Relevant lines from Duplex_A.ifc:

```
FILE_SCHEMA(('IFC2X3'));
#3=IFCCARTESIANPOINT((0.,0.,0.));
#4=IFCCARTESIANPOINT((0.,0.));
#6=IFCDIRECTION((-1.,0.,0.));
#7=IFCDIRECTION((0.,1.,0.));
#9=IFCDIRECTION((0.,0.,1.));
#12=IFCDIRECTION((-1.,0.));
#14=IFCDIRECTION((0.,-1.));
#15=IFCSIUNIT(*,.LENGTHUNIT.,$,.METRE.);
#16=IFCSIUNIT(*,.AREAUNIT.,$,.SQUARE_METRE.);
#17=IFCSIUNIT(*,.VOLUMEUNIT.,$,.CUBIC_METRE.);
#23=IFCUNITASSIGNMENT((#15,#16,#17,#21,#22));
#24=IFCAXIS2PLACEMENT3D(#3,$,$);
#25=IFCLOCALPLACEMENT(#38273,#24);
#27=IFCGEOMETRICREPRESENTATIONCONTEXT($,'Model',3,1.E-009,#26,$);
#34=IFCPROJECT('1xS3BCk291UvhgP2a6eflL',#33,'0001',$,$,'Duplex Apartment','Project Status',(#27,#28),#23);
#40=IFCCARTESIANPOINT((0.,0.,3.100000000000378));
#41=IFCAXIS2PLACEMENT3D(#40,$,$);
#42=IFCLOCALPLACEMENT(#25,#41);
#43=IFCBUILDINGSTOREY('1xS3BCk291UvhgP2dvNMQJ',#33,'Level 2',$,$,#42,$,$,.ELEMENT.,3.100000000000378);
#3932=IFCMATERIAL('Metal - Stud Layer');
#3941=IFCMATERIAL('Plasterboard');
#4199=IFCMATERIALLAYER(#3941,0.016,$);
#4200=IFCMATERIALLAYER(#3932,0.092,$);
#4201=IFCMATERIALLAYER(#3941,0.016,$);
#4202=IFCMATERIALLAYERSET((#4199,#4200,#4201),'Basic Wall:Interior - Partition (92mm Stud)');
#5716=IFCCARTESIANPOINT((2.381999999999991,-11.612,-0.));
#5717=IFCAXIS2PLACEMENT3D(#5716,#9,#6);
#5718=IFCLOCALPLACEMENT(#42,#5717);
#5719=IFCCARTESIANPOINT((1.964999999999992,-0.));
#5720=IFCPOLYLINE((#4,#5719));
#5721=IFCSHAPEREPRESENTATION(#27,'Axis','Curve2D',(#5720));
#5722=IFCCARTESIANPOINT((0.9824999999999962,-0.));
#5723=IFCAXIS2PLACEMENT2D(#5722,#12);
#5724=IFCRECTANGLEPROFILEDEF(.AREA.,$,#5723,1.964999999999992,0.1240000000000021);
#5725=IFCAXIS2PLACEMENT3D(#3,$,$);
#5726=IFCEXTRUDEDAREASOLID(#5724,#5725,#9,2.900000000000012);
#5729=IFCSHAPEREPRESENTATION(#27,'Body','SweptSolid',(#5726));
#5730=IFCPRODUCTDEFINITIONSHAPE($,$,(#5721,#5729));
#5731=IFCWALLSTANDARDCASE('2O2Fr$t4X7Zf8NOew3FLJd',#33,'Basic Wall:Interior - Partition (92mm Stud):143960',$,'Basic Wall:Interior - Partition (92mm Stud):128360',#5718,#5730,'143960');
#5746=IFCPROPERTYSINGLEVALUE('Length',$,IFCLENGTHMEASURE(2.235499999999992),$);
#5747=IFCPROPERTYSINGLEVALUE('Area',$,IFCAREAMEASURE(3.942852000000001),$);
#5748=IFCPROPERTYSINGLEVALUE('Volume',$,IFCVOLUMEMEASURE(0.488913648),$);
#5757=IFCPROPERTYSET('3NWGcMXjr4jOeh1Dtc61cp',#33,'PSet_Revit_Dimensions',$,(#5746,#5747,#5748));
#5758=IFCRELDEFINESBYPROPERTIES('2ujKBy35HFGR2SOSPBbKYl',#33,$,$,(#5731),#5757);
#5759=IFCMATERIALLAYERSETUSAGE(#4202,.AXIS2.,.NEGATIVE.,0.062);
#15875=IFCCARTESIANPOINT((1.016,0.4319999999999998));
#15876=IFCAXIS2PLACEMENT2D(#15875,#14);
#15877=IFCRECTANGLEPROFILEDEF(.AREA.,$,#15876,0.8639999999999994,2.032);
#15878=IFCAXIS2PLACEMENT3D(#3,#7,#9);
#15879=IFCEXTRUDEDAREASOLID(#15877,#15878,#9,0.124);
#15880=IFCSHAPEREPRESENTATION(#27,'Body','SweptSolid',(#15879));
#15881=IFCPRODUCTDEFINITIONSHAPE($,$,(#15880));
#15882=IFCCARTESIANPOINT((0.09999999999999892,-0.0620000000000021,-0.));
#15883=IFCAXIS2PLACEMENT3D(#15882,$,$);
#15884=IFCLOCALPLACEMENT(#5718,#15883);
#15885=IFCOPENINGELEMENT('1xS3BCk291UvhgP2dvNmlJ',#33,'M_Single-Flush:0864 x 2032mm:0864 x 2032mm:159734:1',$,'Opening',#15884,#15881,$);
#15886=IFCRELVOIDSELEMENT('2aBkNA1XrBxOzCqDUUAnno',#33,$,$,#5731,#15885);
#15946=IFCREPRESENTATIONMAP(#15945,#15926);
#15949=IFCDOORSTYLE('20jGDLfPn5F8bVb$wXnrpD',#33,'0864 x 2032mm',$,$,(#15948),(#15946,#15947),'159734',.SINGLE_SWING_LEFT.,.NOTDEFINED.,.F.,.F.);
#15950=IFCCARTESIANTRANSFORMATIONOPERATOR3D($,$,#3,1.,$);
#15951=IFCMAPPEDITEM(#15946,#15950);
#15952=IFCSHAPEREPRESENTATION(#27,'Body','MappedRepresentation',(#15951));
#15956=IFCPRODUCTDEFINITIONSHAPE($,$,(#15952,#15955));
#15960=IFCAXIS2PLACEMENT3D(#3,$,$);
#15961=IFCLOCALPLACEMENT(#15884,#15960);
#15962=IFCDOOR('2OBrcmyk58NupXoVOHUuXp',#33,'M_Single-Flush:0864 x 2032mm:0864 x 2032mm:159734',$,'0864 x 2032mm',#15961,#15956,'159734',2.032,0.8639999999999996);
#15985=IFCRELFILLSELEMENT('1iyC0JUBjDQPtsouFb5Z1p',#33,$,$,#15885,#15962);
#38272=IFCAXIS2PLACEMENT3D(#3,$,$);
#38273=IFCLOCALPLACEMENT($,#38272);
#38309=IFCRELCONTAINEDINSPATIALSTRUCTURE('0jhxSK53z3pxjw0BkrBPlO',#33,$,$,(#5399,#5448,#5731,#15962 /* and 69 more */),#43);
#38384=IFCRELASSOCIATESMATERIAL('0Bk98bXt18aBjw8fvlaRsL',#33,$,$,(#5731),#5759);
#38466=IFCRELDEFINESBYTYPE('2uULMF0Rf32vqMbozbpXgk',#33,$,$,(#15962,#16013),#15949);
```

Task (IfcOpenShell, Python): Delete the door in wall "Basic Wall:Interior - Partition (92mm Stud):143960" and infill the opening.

```python
import ifcopenshell
import ifcopenshell.api.feature
import ifcopenshell.api.pset
import ifcopenshell.api.root
import ifcopenshell.geom
import ifcopenshell.util.element
import ifcopenshell.util.shape
import ifcopenshell.util.unit

model = ifcopenshell.open("Duplex_A.ifc")
area_scale = ifcopenshell.util.unit.calculate_unit_scale(model, "AREAUNIT")
volume_scale = ifcopenshell.util.unit.calculate_unit_scale(model, "VOLUMEUNIT")
settings = ifcopenshell.geom.settings()


def volume(element):
    """Net volume in cubic metres, openings subtracted."""
    shape = ifcopenshell.geom.create_shape(settings, element)
    return ifcopenshell.util.shape.get_volume(shape.geometry)


door = model.by_id(15962)
opening = door.FillsVoids[0].RelatingOpeningElement
wall = opening.VoidsElements[0].RelatingBuildingElement
before = volume(wall)

ifcopenshell.api.root.remove_product(model, product=door)
ifcopenshell.api.feature.remove_feature(model, feature=opening)

after = volume(wall)
thickness = 0.124  # wall thickness in metres

# Update the wall's stored quantities.
pset = model.by_id(ifcopenshell.util.element.get_pset(wall, "PSet_Revit_Dimensions", should_inherit=False)["id"])
ifcopenshell.api.pset.edit_pset(model, pset=pset, properties={
    "Area": model.create_entity("IfcAreaMeasure", after / thickness / area_scale),
    "Volume": model.create_entity("IfcVolumeMeasure", after / volume_scale),
})

print(f"wall volume {before:.3f} -> {after:.3f} m3")

model.write("Duplex_A-out.ifc")
```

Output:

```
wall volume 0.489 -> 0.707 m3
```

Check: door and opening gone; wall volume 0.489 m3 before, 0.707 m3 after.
